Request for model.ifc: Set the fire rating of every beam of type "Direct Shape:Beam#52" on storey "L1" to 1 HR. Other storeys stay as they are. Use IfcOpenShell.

First a look at what the model holds.

```python
import ifcopenshell
import ifcopenshell.util.element

model = ifcopenshell.open("model.ifc")
print(model.schema)
storey = next(s for s in model.by_type("IfcBuildingStorey") if s.Name == "L1")
beams = [e for e in ifcopenshell.util.element.get_decomposition(storey) if e.is_a("IfcBeam")]
seen = {}
for e in beams:
    element_type = ifcopenshell.util.element.get_type(e)
    key = (element_type.Name if element_type != e and element_type else None, ifcopenshell.util.element.get_pset(e, "Pset_BeamCommon", "FireRating"))
    seen[key] = seen.get(key, 0) + 1
for (name, value), count in sorted(seen.items(), key=str):
    print(count, "x", name, "|", value)
```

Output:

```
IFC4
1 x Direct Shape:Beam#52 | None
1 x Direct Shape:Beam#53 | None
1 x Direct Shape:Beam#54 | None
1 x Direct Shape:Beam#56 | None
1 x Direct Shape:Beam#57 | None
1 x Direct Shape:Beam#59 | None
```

```python
import ifcopenshell
import ifcopenshell.api.pset
import ifcopenshell.util.element

model = ifcopenshell.open("model.ifc")

storey = next(s for s in model.by_type("IfcBuildingStorey") if s.Name == "L1")
beams = [e for e in ifcopenshell.util.element.get_decomposition(storey) if e.is_a("IfcBeam")]

count = 0
for e in beams:
    element_type = ifcopenshell.util.element.get_type(e)
    if element_type in (None, e) or element_type.Name != "Direct Shape:Beam#52":
        continue
    # add_pset returns the element's existing set when there is one.
    pset = ifcopenshell.api.pset.add_pset(model, product=e, name="Pset_BeamCommon")
    ifcopenshell.api.pset.edit_pset(model, pset=pset, properties={"FireRating": "1 HR"})
    count += 1

print(count, "beams updated")

model.write("model_edited.ifc")
```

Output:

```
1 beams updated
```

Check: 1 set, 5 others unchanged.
